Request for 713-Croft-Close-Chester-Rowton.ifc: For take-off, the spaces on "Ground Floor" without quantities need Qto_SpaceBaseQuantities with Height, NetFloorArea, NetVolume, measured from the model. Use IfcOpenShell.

First a look at what the model holds.

```python
import ifcopenshell
import ifcopenshell.util.element
import ifcopenshell.util.unit

model = ifcopenshell.open("713-Croft-Close-Chester-Rowton.ifc")
print(model.schema)
for unit_type in ("LENGTHUNIT", "AREAUNIT", "VOLUMEUNIT"):
    print(unit_type, ifcopenshell.util.unit.calculate_unit_scale(model, unit_type))
storey = next(s for s in model.by_type("IfcBuildingStorey") if s.Name == "Ground Floor")
spaces = [e for e in ifcopenshell.util.element.get_decomposition(storey) if e.is_a("IfcSpace")]
for e in sorted(spaces, key=lambda e: e.id()):
    print(e.id(), e.is_a(), e.Name, list(ifcopenshell.util.element.get_psets(e, qtos_only=True)), sep=" | ")
```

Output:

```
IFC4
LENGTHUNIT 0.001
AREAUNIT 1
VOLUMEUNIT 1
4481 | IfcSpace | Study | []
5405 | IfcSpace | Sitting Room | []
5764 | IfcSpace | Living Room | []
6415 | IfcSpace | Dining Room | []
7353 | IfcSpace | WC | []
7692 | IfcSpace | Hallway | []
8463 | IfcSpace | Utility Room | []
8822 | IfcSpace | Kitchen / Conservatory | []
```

```python
import ifcopenshell
import ifcopenshell.api.pset
import ifcopenshell.geom
import ifcopenshell.util.element
import ifcopenshell.util.shape
import ifcopenshell.util.unit

model = ifcopenshell.open("713-Croft-Close-Chester-Rowton.ifc")
unit_scale = ifcopenshell.util.unit.calculate_unit_scale(model)
area_scale = ifcopenshell.util.unit.calculate_unit_scale(model, "AREAUNIT")
volume_scale = ifcopenshell.util.unit.calculate_unit_scale(model, "VOLUMEUNIT")
settings = ifcopenshell.geom.settings()

storey = next(s for s in model.by_type("IfcBuildingStorey") if s.Name == "Ground Floor")
spaces = [e for e in ifcopenshell.util.element.get_decomposition(storey) if e.is_a("IfcSpace")]

for e in sorted(spaces, key=lambda e: e.id()):
    if ifcopenshell.util.element.get_psets(e, qtos_only=True, should_inherit=False):
        continue
    # Geometry comes back in metres, in the element's own axes.
    shape = ifcopenshell.geom.create_shape(settings, e)
    values = {
        "Height": ifcopenshell.util.shape.get_z(shape.geometry) / unit_scale,
        "NetFloorArea": ifcopenshell.util.shape.get_footprint_area(shape.geometry) / area_scale,
        "NetVolume": ifcopenshell.util.shape.get_volume(shape.geometry) / volume_scale,
    }
    qto = ifcopenshell.api.pset.add_qto(model, product=e, name="Qto_SpaceBaseQuantities")
    ifcopenshell.api.pset.edit_qto(model, qto=qto, properties=values)
    print(e.id(), {k: round(v, 3) for k, v in values.items()})

model.write("713-Croft-Close-Chester-Rowton-out.ifc")
```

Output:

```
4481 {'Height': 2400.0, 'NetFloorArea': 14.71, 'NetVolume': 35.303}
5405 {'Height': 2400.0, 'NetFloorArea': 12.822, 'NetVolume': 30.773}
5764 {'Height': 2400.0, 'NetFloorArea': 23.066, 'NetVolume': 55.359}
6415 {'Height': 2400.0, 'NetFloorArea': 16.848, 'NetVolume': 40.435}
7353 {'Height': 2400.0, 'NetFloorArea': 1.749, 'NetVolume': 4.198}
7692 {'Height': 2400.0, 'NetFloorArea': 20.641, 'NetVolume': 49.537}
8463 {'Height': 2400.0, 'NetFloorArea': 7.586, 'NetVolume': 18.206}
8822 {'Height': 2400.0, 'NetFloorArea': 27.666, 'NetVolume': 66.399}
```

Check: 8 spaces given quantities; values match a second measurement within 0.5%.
